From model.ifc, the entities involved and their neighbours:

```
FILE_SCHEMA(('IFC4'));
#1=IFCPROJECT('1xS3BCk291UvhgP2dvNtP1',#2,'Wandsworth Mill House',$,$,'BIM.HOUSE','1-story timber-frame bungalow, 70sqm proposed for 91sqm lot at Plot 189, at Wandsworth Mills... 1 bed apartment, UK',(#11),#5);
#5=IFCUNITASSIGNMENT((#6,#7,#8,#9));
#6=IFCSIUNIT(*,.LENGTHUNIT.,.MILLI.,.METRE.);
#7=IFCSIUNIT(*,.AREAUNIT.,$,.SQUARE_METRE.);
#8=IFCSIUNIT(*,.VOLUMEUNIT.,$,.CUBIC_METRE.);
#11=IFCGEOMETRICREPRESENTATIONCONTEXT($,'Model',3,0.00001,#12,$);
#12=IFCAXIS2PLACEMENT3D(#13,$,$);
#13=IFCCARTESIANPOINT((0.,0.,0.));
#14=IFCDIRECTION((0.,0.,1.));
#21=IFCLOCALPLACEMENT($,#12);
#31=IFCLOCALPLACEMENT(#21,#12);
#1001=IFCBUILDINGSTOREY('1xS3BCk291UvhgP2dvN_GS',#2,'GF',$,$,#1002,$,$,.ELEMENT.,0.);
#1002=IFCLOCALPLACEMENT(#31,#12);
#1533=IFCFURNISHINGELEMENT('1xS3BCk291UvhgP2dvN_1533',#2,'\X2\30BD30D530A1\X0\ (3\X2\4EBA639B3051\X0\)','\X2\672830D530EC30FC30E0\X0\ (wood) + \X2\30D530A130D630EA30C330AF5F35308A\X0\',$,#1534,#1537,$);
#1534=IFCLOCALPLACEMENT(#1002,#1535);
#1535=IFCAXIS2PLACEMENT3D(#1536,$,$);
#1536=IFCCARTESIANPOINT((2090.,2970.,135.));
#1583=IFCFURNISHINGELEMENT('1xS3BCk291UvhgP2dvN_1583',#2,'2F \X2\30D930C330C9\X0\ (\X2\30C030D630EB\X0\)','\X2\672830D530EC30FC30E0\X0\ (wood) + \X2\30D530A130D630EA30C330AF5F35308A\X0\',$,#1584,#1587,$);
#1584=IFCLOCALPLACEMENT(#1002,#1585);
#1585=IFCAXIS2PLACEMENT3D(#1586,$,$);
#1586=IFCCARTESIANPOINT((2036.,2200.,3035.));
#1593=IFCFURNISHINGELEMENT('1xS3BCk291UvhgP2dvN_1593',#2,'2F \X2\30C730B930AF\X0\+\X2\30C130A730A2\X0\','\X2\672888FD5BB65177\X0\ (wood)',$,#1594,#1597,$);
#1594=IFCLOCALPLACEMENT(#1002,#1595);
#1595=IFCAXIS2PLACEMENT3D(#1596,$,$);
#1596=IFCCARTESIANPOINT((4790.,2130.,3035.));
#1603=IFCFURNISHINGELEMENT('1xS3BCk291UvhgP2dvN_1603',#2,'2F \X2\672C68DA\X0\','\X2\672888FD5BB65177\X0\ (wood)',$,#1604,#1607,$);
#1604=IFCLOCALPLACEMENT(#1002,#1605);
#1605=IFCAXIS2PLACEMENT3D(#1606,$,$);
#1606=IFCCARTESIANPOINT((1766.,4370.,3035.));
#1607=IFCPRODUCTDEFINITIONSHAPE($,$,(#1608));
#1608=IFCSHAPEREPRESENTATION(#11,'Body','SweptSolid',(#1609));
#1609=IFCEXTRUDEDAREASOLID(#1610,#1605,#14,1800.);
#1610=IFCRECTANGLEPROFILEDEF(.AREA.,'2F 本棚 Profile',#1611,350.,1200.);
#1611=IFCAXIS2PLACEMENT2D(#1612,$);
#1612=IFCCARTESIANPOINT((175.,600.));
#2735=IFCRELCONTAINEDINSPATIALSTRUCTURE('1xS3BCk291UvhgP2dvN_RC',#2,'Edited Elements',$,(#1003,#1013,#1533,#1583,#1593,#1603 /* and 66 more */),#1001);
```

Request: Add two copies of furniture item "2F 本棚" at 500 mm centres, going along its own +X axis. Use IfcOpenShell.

```python
import ifcopenshell
import ifcopenshell.api.geometry
import ifcopenshell.api.root
import ifcopenshell.util.element
import ifcopenshell.util.placement
import ifcopenshell.util.unit

model = ifcopenshell.open("model.ifc")
unit_scale = ifcopenshell.util.unit.calculate_unit_scale(model)


def reuse_history(source, copy):
    """copy_class also copies each property set's owner history, people and application; keep the originals."""
    for rel in copy.IsDefinedBy:
        if rel.is_a("IfcRelDefinesByProperties") and (history := rel.RelatingPropertyDefinition.OwnerHistory):
            rel.RelatingPropertyDefinition.OwnerHistory = source.OwnerHistory
            ifcopenshell.util.element.remove_deep2(model, history)


source = model.by_id(1603)
base = ifcopenshell.util.placement.get_local_placement(source.ObjectPlacement)
step = base[:3, 0] * 0.5 / unit_scale

for i in range(1, 3):
    copy = ifcopenshell.api.root.copy_class(model, product=source)
    copy.Representation = ifcopenshell.util.element.copy_deep(
        model, source.Representation, exclude=["IfcGeometricRepresentationContext", "IfcRepresentationMap"]
    )
    reuse_history(source, copy)
    matrix = base.copy()
    matrix[:3, 3] += i * step
    print("added at", matrix[:3, 3].round(3) + 0.0)
    ifcopenshell.api.geometry.edit_object_placement(model, product=copy, matrix=matrix, is_si=False)

model.write("model-out.ifc")
```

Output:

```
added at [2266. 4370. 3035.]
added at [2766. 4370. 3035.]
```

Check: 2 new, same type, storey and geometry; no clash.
